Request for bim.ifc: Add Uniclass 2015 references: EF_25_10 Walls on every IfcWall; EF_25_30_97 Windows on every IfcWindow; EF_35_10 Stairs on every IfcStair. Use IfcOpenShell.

First a look at what the model holds.

```python
import ifcopenshell

model = ifcopenshell.open("bim.ifc")
print(model.schema)
print("classifications:", [c.Name for c in model.by_type("IfcClassification")])
for ifc_class in ("IfcDoor", "IfcRoof", "IfcStair", "IfcWall", "IfcWindow"):
    print(ifc_class, len(model.by_type(ifc_class)))
```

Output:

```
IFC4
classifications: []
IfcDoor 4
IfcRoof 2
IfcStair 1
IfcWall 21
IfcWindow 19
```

```python
import ifcopenshell
import ifcopenshell.api.classification

model = ifcopenshell.open("bim.ifc")

system = ifcopenshell.api.classification.add_classification(model, classification="Uniclass 2015")

codes = {
    "IfcWall": ("EF_25_10", "Walls"),
    "IfcWindow": ("EF_25_30_97", "Windows"),
    "IfcStair": ("EF_35_10", "Stairs"),
}
for ifc_class, (code, name) in codes.items():
    products = model.by_type(ifc_class)
    ifcopenshell.api.classification.add_reference(
        model, products=products, classification=system, identification=code, name=name
    )
    print(code, len(products))

model.write("bim_edited.ifc")
```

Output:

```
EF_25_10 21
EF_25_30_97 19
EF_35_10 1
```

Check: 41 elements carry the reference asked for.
